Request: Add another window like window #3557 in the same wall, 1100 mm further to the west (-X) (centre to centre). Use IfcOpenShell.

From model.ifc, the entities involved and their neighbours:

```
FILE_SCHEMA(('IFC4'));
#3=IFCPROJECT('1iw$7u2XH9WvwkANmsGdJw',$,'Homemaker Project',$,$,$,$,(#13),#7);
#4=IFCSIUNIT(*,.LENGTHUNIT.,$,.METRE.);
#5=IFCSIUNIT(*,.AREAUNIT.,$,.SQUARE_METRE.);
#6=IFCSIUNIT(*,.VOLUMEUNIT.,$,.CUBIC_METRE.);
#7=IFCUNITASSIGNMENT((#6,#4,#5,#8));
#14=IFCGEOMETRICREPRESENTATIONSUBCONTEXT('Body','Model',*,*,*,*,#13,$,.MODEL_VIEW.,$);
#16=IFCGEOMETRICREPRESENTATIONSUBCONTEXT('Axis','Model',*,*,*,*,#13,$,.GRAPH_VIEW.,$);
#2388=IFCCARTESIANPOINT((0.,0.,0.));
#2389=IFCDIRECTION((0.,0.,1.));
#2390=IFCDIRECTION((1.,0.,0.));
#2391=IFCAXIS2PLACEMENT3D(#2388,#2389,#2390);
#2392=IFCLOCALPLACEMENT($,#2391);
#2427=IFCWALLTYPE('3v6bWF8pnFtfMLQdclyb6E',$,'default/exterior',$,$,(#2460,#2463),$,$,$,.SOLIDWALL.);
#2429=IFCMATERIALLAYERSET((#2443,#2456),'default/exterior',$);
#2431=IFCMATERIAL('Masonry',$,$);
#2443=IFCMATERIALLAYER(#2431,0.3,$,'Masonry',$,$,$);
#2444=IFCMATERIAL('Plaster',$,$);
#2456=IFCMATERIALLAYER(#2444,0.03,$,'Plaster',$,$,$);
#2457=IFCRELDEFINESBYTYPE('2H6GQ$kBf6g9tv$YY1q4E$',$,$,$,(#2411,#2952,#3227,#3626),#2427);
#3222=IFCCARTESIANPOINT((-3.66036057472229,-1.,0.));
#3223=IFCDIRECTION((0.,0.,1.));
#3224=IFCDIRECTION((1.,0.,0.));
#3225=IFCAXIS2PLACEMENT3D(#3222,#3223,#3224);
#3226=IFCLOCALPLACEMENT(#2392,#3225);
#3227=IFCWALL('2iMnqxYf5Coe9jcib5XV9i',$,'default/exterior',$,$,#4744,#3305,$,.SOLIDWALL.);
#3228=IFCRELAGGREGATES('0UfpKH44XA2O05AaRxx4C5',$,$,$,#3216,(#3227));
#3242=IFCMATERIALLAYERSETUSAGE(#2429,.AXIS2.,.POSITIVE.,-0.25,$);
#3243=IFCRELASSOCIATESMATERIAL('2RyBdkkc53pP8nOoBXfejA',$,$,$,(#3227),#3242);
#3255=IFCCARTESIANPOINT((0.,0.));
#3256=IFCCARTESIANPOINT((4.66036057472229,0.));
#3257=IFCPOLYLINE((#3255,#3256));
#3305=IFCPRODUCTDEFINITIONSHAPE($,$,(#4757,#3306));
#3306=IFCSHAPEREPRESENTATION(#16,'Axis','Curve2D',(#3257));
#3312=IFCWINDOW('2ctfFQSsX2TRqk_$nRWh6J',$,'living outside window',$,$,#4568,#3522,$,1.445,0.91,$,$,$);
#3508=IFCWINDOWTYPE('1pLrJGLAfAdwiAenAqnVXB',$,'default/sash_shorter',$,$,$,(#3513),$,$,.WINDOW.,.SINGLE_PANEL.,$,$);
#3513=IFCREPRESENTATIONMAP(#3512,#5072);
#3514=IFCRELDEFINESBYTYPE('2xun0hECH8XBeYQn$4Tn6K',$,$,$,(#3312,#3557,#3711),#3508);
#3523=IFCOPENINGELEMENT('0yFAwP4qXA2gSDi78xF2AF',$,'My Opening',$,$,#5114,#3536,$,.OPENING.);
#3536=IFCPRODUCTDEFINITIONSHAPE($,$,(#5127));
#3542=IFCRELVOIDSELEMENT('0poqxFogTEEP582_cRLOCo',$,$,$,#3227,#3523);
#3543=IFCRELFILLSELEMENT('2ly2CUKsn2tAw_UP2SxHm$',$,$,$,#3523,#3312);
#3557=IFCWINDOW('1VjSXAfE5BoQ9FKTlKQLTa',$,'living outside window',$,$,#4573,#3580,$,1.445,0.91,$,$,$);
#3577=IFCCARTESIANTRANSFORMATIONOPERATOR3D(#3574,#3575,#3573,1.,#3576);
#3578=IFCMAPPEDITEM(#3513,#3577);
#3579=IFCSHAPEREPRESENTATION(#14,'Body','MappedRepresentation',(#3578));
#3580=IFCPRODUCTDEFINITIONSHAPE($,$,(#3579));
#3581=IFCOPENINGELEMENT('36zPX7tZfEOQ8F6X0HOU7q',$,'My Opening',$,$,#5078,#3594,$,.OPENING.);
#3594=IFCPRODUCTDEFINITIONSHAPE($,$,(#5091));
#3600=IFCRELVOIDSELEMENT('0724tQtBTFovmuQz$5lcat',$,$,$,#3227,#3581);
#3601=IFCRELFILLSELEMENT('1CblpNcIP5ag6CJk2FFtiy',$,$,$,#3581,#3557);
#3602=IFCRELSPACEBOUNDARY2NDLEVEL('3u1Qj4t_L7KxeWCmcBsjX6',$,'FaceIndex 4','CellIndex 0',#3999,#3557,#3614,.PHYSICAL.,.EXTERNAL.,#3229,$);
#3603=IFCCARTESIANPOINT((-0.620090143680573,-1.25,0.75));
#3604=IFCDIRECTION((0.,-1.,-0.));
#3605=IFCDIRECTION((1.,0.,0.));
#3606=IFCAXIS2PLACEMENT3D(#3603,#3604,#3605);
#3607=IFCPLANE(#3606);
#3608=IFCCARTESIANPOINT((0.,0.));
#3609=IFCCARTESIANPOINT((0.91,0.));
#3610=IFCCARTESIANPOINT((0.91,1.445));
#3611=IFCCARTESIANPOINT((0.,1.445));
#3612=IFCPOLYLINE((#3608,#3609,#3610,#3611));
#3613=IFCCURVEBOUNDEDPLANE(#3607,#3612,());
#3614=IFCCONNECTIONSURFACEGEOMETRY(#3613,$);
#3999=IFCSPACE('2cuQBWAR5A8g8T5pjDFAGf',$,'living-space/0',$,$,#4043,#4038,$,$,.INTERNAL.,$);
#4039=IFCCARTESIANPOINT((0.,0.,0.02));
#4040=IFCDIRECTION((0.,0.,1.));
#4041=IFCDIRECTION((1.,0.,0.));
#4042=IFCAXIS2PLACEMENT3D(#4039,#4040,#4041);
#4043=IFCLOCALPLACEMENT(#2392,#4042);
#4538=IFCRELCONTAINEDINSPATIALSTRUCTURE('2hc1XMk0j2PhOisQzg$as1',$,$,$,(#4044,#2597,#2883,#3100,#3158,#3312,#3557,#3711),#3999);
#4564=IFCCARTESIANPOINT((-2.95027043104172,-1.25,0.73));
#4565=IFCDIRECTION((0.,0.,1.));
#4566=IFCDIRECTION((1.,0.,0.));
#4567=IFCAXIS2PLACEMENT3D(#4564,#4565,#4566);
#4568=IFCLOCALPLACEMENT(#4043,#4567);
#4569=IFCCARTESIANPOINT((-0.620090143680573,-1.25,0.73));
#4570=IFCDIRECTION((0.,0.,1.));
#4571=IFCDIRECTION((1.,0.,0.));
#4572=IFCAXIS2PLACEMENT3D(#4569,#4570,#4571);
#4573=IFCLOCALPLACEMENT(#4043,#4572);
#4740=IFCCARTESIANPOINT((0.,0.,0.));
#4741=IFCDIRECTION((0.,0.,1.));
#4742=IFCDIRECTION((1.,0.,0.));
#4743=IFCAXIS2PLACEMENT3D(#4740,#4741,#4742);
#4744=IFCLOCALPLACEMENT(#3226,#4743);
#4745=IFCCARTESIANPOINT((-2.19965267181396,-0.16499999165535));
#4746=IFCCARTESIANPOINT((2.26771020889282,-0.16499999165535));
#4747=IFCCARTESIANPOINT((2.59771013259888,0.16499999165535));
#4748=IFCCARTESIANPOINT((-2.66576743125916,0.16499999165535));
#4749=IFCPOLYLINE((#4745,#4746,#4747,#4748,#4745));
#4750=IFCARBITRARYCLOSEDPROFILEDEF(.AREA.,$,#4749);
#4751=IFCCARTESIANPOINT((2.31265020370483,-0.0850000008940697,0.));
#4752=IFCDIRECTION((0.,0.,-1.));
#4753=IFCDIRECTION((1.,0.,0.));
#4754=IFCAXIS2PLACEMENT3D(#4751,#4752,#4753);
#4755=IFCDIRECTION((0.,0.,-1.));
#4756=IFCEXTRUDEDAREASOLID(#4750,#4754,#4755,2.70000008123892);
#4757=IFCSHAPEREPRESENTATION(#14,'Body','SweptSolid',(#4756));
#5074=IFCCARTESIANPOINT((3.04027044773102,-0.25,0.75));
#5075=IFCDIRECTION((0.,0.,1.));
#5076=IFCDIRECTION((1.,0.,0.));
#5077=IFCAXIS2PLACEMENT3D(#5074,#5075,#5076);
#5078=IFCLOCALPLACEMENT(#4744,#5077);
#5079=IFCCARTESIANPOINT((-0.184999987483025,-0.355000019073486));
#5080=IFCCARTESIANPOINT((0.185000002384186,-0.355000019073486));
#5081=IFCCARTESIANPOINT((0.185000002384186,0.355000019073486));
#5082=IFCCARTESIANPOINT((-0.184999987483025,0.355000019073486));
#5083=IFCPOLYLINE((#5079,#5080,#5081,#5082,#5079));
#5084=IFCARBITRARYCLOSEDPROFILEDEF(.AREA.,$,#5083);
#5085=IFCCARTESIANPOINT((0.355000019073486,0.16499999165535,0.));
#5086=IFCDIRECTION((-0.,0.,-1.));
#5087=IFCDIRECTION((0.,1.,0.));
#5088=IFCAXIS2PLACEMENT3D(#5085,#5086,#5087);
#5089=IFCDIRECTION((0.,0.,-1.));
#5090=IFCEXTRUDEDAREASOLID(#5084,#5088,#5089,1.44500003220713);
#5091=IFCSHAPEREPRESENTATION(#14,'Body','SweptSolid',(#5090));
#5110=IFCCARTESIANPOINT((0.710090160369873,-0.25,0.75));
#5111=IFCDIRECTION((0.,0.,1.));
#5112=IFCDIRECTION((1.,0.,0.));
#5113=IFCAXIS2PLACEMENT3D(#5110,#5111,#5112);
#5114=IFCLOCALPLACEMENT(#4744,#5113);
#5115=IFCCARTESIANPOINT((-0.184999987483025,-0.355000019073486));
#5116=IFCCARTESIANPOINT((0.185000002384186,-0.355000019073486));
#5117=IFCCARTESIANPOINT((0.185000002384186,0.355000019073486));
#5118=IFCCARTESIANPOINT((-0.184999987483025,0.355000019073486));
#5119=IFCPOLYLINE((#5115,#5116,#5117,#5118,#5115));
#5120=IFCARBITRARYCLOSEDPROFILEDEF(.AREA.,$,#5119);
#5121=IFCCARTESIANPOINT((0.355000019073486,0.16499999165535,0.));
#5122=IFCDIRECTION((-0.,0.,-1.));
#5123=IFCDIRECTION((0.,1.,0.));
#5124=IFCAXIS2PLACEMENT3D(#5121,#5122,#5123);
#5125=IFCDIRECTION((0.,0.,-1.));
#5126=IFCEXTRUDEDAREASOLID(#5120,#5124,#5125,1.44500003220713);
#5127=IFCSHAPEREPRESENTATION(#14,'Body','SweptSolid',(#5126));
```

```python
import numpy as np
import ifcopenshell
import ifcopenshell.api.feature
import ifcopenshell.api.geometry
import ifcopenshell.api.root
import ifcopenshell.geom
import ifcopenshell.util.element
import ifcopenshell.util.placement
import ifcopenshell.util.shape

model = ifcopenshell.open("model.ifc")
settings = ifcopenshell.geom.settings()


def volume(element):
    """Net volume in cubic metres, openings subtracted."""
    shape = ifcopenshell.geom.create_shape(settings, element)
    return ifcopenshell.util.shape.get_volume(shape.geometry)


window = model.by_id(3557)
opening = window.FillsVoids[0].RelatingOpeningElement
wall = opening.VoidsElements[0].RelatingBuildingElement
before = volume(wall)
shift = ifcopenshell.util.placement.get_local_placement(wall.ObjectPlacement)[:3, 0] * -1.1

# copy_class copies the void relationship, type, container and properties, but no geometry.
new_opening = ifcopenshell.api.root.copy_class(model, product=opening)
new_opening.Representation = ifcopenshell.util.element.copy_deep(
    model, opening.Representation, exclude=["IfcGeometricRepresentationContext", "IfcRepresentationMap"]
)
new_window = ifcopenshell.api.root.copy_class(model, product=window)
new_window.Representation = ifcopenshell.util.element.copy_deep(
    model, window.Representation, exclude=["IfcGeometricRepresentationContext", "IfcRepresentationMap"]
)
ifcopenshell.api.feature.add_filling(model, opening=new_opening, element=new_window)

for old, new in ((opening, new_opening), (window, new_window)):
    matrix = ifcopenshell.util.placement.get_local_placement(old.ObjectPlacement)
    matrix[:3, 3] += shift
    ifcopenshell.api.geometry.edit_object_placement(model, product=new, matrix=matrix, is_si=False)

# The copied space boundaries still share their surfaces with the original.
for rel in new_window.ProvidesBoundaries:
    if rel.ConnectionGeometry:
        rel.ConnectionGeometry = ifcopenshell.util.element.copy_deep(model, rel.ConnectionGeometry)

# Space boundary surfaces are stored in each space's coordinates; move them too.
for rel in new_window.ProvidesBoundaries:
    if not rel.ConnectionGeometry:
        continue
    surface = rel.ConnectionGeometry.SurfaceOnRelatingElement.BasisSurface
    space_matrix = ifcopenshell.util.placement.get_local_placement(rel.RelatingSpace.ObjectPlacement)
    point = np.array(surface.Position.Location.Coordinates) + space_matrix[:3, :3].T @ shift
    surface.Position = model.createIfcAxis2Placement3D(
        model.createIfcCartesianPoint(point.tolist()), surface.Position.Axis, surface.Position.RefDirection
    )

after = volume(wall)

print(f"wall volume {before:.3f} -> {after:.3f} m3")

model.write("model_v2.ifc")
```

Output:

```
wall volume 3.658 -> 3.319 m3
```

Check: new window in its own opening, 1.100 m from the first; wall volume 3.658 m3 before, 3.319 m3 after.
